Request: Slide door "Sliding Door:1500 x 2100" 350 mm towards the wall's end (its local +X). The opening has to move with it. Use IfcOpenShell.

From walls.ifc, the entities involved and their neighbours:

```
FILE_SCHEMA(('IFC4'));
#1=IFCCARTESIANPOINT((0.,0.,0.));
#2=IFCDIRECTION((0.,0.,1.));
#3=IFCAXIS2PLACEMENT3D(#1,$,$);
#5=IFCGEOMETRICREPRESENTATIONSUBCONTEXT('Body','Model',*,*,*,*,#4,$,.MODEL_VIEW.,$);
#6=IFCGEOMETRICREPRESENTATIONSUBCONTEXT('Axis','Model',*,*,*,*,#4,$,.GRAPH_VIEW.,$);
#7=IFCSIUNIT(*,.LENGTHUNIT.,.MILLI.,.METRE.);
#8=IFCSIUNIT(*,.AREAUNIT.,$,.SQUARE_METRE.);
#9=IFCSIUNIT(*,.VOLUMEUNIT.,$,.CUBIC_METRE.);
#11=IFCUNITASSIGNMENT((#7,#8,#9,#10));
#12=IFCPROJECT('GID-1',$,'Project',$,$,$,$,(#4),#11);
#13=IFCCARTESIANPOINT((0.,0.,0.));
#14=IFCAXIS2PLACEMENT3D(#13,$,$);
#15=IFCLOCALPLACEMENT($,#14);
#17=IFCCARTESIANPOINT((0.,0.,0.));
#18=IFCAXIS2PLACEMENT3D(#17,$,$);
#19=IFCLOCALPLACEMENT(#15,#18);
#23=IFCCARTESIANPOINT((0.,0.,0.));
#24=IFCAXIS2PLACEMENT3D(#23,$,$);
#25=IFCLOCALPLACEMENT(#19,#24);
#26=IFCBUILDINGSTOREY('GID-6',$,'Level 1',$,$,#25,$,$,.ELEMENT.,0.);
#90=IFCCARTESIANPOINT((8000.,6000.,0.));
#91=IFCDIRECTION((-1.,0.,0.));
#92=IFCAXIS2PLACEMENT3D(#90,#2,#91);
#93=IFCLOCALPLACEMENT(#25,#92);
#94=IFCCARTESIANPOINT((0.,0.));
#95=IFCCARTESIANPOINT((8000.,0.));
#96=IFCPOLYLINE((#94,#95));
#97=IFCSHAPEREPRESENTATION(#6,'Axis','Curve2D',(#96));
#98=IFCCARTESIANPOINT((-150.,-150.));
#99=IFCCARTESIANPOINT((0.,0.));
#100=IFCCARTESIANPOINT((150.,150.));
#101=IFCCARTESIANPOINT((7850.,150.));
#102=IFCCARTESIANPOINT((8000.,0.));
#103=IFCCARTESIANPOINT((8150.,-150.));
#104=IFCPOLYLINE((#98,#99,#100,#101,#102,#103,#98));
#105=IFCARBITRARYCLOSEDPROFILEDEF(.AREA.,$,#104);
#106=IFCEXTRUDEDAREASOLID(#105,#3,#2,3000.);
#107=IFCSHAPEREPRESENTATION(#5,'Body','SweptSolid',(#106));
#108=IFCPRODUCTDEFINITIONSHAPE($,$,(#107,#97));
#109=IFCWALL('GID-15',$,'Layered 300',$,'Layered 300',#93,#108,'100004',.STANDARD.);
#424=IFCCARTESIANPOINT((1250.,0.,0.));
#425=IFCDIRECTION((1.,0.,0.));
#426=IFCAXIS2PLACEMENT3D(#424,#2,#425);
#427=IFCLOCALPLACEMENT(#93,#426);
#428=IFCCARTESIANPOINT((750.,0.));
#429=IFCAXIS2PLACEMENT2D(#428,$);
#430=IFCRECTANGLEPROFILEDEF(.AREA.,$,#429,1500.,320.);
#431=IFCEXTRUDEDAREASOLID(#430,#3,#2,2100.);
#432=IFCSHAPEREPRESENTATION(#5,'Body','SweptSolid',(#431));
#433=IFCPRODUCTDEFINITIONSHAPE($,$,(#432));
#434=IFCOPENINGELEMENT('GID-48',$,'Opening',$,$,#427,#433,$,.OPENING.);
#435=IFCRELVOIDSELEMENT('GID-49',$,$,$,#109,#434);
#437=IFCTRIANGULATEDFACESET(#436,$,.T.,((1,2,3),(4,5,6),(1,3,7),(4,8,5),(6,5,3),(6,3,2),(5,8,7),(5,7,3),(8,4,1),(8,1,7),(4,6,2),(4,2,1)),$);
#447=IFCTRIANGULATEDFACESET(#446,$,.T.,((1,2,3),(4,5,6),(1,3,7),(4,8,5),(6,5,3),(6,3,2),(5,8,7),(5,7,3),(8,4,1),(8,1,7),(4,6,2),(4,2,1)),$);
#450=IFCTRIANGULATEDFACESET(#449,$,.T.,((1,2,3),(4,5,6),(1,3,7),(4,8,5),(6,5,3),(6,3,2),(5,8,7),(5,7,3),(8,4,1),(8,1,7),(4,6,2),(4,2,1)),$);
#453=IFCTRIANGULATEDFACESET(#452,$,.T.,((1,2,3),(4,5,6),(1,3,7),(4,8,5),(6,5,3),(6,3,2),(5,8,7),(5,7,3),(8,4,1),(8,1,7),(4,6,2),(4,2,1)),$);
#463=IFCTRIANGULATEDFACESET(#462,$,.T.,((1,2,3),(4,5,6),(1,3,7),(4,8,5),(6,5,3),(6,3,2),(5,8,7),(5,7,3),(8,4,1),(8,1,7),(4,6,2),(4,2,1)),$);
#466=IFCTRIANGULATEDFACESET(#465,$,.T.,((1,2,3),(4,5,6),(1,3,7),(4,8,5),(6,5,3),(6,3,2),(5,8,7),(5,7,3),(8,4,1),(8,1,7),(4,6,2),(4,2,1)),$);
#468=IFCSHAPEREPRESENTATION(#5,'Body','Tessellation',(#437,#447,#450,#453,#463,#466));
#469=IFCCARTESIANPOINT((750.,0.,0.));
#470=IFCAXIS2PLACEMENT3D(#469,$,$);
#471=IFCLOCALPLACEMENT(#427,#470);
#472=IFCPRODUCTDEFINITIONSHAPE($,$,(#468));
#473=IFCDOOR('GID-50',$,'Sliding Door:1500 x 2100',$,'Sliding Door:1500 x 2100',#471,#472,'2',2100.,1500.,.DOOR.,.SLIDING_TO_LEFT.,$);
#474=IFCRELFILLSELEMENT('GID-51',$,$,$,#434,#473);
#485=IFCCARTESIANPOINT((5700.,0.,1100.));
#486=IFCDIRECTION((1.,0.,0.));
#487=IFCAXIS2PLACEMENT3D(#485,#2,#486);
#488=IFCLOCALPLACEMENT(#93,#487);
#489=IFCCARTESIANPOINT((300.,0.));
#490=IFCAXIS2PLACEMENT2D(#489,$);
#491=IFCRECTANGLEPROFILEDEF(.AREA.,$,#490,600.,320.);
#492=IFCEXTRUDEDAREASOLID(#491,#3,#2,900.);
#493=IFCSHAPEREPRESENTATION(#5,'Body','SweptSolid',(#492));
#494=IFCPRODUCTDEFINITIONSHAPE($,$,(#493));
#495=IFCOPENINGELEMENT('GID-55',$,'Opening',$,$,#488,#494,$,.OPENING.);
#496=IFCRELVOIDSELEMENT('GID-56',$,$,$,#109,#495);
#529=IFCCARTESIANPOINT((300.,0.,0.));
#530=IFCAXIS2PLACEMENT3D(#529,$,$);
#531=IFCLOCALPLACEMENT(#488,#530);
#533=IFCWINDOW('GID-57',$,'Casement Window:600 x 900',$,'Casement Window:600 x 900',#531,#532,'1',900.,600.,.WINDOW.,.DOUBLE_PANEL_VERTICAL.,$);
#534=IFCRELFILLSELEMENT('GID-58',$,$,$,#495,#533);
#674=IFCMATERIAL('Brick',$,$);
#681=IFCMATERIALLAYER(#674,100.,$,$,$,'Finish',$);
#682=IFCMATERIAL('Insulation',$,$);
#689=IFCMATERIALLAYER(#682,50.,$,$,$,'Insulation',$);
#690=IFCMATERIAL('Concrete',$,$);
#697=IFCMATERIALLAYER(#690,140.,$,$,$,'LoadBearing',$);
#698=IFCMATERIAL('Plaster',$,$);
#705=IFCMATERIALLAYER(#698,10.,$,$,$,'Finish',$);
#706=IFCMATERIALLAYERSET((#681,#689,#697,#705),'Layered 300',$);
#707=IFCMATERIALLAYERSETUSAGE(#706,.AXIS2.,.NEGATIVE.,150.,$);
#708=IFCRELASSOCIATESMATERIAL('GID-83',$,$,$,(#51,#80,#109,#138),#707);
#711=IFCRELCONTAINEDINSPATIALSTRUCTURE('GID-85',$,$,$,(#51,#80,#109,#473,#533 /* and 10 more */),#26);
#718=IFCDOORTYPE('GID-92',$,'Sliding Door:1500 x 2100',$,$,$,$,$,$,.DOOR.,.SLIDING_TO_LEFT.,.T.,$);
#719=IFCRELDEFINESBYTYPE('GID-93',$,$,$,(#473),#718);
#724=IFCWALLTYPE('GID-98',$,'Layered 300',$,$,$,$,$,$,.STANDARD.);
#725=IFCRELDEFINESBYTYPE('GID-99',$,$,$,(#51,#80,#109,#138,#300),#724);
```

```python
import ifcopenshell
import ifcopenshell.api.geometry
import ifcopenshell.util.placement

model = ifcopenshell.open("walls.ifc")

door = model.by_guid("GID-50")
opening = door.FillsVoids[0].RelatingOpeningElement
wall = opening.VoidsElements[0].RelatingBuildingElement

wall_matrix = ifcopenshell.util.placement.get_local_placement(wall.ObjectPlacement)
shift = wall_matrix[:3, 0] * 350.0
before = ifcopenshell.util.placement.get_local_placement(door.ObjectPlacement)[:3, 3].copy()

# The door is placed relative to its opening, so it follows when the opening moves.
matrix = ifcopenshell.util.placement.get_local_placement(opening.ObjectPlacement)
matrix[:3, 3] += shift
ifcopenshell.api.geometry.edit_object_placement(
    model, product=opening, matrix=matrix, is_si=False, should_transform_children=True
)

after = ifcopenshell.util.placement.get_local_placement(door.ObjectPlacement)[:3, 3]
print("door moved by", (after - before).round(3) + 0.0)

model.write("walls_v2.ifc")
```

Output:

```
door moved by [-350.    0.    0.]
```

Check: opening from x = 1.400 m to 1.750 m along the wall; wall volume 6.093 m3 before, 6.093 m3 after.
